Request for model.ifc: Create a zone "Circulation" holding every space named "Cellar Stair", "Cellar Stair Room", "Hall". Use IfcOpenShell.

First a look at what the model holds.

```python
import ifcopenshell

model = ifcopenshell.open("model.ifc")
print(model.schema)
seen = {}
for space in model.by_type("IfcSpace"):
    seen[space.LongName] = seen.get(space.LongName, 0) + 1
for name, count in sorted(seen.items(), key=str):
    print(count, "x", name)
print("zones:", [z.Name for z in model.by_type("IfcZone")][:20])
```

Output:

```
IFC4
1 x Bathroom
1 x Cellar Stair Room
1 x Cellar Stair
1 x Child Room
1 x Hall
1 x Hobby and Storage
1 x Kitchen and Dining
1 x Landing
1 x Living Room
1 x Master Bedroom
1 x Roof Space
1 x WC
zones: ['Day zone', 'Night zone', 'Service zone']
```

```python
import ifcopenshell
import ifcopenshell.api.group
import ifcopenshell.api.root

model = ifcopenshell.open("model.ifc")

names = {"Cellar Stair", "Cellar Stair Room", "Hall"}
spaces = [s for s in model.by_type("IfcSpace") if s.LongName in names]

zone = ifcopenshell.api.root.create_entity(model, ifc_class="IfcZone", name="Circulation")
ifcopenshell.api.group.assign_group(model, products=spaces, group=zone)
print(len(spaces), "spaces in", zone.Name)

model.write("model-out.ifc")
```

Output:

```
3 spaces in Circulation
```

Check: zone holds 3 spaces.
